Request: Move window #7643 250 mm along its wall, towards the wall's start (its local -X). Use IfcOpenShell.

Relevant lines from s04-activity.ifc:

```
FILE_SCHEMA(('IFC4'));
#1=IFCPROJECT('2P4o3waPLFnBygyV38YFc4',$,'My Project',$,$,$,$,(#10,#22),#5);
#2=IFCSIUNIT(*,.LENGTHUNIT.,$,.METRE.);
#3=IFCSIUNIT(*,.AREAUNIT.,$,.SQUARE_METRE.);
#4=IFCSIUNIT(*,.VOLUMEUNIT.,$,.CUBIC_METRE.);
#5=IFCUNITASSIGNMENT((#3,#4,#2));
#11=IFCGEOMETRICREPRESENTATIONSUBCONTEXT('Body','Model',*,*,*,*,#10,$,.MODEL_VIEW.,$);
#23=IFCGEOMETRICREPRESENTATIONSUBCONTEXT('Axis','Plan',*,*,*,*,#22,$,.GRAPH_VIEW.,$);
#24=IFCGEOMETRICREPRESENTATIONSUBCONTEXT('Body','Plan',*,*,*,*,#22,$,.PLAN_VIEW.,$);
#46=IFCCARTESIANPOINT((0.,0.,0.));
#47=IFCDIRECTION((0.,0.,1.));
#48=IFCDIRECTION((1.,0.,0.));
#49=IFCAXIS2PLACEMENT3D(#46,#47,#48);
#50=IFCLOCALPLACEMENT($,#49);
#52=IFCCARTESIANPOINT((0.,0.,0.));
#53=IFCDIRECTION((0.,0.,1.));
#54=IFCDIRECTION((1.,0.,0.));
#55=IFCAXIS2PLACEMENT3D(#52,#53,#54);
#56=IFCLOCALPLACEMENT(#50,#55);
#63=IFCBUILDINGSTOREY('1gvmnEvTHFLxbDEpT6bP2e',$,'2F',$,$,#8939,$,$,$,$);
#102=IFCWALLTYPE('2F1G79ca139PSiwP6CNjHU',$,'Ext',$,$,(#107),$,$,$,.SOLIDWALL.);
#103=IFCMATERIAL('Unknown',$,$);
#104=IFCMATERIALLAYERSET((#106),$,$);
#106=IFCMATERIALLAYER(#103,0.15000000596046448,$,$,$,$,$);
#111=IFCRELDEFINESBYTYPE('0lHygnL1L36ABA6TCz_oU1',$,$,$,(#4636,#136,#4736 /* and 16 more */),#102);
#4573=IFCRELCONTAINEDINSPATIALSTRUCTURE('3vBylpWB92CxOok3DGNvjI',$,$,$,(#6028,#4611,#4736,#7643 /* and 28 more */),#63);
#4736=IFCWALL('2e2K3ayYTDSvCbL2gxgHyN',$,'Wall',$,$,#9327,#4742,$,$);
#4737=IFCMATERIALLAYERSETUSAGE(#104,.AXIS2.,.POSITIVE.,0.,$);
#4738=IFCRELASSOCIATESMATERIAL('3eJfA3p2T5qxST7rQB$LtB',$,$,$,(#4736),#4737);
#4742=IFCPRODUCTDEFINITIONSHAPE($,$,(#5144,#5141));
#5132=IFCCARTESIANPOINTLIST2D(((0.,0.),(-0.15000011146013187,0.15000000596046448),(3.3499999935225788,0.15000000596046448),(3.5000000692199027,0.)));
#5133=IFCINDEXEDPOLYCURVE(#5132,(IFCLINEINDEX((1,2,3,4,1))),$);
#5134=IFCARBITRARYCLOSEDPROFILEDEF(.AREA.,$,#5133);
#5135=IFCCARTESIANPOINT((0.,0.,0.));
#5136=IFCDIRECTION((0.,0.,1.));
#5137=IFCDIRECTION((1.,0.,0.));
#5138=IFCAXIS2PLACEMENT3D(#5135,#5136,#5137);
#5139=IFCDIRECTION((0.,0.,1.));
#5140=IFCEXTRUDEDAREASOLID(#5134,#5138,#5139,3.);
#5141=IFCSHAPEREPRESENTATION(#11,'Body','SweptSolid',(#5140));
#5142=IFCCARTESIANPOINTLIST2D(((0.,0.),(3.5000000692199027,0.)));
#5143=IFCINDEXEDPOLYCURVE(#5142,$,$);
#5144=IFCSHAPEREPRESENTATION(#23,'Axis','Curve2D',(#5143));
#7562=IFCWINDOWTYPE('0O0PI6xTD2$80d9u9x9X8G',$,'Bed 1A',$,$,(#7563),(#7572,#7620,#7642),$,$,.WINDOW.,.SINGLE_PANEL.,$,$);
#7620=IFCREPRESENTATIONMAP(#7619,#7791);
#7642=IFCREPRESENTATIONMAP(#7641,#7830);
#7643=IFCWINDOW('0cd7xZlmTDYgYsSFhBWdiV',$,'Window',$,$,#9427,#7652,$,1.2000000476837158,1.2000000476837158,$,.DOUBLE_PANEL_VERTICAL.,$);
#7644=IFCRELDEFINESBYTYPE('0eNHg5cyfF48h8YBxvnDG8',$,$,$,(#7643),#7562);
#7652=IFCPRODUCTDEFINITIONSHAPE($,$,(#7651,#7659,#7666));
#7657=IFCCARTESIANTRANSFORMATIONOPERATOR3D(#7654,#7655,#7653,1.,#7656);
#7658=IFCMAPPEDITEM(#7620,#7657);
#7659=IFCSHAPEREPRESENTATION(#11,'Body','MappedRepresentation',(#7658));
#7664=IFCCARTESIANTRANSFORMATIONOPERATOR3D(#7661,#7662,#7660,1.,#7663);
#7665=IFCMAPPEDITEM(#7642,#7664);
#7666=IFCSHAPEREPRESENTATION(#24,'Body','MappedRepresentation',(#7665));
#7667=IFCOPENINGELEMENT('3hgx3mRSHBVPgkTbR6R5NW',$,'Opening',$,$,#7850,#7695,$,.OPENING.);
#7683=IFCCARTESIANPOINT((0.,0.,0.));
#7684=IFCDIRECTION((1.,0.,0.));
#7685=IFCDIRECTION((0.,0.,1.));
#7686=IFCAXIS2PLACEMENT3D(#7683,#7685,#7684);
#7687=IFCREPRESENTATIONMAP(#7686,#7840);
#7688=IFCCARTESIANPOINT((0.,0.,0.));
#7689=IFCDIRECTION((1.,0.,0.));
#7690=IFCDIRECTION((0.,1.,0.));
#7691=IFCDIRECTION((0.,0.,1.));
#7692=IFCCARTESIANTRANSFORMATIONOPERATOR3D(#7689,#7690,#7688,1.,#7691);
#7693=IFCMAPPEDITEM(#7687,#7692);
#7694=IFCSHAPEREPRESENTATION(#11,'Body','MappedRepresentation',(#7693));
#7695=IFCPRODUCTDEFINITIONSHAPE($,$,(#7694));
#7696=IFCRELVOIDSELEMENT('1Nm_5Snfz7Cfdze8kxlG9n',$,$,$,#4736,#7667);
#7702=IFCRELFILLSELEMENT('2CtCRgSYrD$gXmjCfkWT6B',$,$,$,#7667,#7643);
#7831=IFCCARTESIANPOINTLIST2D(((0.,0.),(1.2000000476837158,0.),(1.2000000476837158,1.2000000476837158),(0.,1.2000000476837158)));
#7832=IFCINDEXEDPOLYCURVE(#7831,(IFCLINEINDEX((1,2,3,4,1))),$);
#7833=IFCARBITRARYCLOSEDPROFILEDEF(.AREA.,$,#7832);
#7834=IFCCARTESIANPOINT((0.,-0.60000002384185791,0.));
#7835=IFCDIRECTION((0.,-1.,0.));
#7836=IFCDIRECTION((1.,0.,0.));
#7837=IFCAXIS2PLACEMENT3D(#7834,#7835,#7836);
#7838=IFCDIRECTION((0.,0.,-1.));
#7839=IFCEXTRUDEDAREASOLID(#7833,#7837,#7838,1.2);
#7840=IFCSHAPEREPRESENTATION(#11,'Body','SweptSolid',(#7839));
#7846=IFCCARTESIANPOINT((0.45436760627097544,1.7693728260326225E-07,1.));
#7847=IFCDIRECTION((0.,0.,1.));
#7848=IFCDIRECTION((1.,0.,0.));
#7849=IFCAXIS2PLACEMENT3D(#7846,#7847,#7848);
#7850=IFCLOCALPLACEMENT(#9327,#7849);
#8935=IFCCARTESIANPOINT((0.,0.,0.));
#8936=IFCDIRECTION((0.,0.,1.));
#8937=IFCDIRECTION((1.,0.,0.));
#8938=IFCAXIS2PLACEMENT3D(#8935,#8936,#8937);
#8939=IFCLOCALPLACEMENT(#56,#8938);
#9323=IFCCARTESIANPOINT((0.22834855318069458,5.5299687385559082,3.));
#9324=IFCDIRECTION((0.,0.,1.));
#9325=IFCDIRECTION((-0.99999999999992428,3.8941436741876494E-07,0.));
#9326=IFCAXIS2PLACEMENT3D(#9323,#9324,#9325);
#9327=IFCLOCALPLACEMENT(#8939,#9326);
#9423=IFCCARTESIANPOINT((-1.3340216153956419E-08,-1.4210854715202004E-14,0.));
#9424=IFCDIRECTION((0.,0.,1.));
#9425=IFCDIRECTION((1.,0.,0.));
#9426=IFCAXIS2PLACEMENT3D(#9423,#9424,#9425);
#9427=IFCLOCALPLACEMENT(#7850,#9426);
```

```python
import ifcopenshell
import ifcopenshell.api.geometry
import ifcopenshell.util.placement
import ifcopenshell.util.unit

model = ifcopenshell.open("s04-activity.ifc")
unit_scale = ifcopenshell.util.unit.calculate_unit_scale(model)

window = model.by_id(7643)
opening = window.FillsVoids[0].RelatingOpeningElement
wall = opening.VoidsElements[0].RelatingBuildingElement

wall_matrix = ifcopenshell.util.placement.get_local_placement(wall.ObjectPlacement)
shift = wall_matrix[:3, 0] * -0.25 / unit_scale
before = ifcopenshell.util.placement.get_local_placement(window.ObjectPlacement)[:3, 3].copy()

# The window is placed relative to its opening, so it follows when the opening moves.
matrix = ifcopenshell.util.placement.get_local_placement(opening.ObjectPlacement)
matrix[:3, 3] += shift
ifcopenshell.api.geometry.edit_object_placement(
    model, product=opening, matrix=matrix, is_si=False, should_transform_children=True
)

after = ifcopenshell.util.placement.get_local_placement(window.ObjectPlacement)[:3, 3]
print("window moved by", (after - before).round(3) + 0.0)

model.write("s04-activity_v2.ifc")
```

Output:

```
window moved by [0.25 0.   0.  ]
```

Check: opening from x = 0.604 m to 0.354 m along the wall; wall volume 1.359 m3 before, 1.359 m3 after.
